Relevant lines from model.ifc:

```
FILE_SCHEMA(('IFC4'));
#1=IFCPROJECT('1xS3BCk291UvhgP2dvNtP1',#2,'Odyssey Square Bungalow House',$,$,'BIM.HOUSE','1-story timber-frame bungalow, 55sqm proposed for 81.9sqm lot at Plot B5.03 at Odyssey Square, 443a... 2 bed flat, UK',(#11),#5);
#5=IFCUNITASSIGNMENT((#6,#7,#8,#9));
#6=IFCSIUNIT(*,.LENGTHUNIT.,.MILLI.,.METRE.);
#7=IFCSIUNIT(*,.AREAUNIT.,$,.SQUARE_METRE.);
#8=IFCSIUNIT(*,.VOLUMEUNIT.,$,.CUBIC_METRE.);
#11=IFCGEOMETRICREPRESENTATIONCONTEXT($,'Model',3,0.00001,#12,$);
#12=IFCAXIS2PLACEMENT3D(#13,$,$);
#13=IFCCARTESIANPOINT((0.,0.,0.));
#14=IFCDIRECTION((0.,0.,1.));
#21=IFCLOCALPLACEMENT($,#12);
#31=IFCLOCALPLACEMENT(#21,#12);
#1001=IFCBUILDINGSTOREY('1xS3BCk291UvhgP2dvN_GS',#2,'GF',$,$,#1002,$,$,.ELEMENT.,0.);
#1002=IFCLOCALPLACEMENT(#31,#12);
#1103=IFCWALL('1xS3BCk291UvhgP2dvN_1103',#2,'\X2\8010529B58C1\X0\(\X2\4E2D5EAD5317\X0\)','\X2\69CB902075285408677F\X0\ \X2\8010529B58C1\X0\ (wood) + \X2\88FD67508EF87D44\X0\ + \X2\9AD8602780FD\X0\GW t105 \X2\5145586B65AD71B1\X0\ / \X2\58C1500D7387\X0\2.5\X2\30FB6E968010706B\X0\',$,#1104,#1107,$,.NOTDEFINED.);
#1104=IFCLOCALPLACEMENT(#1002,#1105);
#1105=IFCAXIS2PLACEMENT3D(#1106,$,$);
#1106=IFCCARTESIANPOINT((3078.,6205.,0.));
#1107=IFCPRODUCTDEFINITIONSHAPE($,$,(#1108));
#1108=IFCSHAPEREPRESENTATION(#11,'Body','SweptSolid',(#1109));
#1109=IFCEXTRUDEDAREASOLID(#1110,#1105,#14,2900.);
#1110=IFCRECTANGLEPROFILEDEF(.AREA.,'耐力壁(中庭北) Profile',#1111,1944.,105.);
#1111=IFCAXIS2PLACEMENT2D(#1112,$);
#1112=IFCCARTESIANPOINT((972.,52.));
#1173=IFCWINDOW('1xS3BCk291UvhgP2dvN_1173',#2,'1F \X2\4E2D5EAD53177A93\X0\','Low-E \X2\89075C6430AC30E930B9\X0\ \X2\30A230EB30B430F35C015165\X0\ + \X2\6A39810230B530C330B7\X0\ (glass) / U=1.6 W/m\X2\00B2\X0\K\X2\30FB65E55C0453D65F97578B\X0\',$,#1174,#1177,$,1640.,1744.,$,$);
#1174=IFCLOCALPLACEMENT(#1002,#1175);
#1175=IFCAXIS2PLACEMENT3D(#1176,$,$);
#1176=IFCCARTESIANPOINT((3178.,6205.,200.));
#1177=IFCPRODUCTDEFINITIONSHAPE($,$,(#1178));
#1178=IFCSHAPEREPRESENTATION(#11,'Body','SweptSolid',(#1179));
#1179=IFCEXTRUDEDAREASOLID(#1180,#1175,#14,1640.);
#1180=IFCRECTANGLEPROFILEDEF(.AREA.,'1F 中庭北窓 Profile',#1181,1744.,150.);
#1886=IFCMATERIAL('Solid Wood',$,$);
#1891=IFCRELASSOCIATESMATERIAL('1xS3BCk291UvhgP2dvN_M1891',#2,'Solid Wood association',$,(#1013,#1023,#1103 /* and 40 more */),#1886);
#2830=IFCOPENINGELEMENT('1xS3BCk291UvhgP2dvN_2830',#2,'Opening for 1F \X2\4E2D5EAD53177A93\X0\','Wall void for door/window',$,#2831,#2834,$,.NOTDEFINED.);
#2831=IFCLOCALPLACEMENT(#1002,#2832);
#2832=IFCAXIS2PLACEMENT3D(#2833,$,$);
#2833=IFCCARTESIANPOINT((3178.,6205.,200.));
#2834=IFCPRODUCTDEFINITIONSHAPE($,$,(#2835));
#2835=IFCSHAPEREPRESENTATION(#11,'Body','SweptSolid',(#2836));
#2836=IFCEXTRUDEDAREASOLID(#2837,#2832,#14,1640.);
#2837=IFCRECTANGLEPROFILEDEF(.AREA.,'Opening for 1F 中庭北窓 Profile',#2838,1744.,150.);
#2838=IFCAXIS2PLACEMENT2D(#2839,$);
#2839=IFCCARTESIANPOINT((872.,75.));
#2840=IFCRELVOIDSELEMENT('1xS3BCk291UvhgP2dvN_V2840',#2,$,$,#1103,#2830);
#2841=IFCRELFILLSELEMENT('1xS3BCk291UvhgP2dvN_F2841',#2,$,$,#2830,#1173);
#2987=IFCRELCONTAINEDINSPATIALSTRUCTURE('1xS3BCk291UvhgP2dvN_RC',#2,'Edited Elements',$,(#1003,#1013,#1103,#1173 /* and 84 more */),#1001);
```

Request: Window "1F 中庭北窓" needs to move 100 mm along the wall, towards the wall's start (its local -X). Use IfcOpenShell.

```python
import ifcopenshell
import ifcopenshell.api.geometry
import ifcopenshell.util.placement

model = ifcopenshell.open("model.ifc")

window = model.by_id(1173)
opening = window.FillsVoids[0].RelatingOpeningElement
wall = opening.VoidsElements[0].RelatingBuildingElement

wall_matrix = ifcopenshell.util.placement.get_local_placement(wall.ObjectPlacement)
shift = wall_matrix[:3, 0] * -100.0
before = ifcopenshell.util.placement.get_local_placement(window.ObjectPlacement)[:3, 3].copy()

# The window is not placed relative to its opening, so move both.
for product in (opening, window):
    matrix = ifcopenshell.util.placement.get_local_placement(product.ObjectPlacement)
    matrix[:3, 3] += shift
    ifcopenshell.api.geometry.edit_object_placement(model, product=product, matrix=matrix, is_si=False)

after = ifcopenshell.util.placement.get_local_placement(window.ObjectPlacement)[:3, 3]
print("window moved by", (after - before).round(3) + 0.0)

model.write("model_updated.ifc")
```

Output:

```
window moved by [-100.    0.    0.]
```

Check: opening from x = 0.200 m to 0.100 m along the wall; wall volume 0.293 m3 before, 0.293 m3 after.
